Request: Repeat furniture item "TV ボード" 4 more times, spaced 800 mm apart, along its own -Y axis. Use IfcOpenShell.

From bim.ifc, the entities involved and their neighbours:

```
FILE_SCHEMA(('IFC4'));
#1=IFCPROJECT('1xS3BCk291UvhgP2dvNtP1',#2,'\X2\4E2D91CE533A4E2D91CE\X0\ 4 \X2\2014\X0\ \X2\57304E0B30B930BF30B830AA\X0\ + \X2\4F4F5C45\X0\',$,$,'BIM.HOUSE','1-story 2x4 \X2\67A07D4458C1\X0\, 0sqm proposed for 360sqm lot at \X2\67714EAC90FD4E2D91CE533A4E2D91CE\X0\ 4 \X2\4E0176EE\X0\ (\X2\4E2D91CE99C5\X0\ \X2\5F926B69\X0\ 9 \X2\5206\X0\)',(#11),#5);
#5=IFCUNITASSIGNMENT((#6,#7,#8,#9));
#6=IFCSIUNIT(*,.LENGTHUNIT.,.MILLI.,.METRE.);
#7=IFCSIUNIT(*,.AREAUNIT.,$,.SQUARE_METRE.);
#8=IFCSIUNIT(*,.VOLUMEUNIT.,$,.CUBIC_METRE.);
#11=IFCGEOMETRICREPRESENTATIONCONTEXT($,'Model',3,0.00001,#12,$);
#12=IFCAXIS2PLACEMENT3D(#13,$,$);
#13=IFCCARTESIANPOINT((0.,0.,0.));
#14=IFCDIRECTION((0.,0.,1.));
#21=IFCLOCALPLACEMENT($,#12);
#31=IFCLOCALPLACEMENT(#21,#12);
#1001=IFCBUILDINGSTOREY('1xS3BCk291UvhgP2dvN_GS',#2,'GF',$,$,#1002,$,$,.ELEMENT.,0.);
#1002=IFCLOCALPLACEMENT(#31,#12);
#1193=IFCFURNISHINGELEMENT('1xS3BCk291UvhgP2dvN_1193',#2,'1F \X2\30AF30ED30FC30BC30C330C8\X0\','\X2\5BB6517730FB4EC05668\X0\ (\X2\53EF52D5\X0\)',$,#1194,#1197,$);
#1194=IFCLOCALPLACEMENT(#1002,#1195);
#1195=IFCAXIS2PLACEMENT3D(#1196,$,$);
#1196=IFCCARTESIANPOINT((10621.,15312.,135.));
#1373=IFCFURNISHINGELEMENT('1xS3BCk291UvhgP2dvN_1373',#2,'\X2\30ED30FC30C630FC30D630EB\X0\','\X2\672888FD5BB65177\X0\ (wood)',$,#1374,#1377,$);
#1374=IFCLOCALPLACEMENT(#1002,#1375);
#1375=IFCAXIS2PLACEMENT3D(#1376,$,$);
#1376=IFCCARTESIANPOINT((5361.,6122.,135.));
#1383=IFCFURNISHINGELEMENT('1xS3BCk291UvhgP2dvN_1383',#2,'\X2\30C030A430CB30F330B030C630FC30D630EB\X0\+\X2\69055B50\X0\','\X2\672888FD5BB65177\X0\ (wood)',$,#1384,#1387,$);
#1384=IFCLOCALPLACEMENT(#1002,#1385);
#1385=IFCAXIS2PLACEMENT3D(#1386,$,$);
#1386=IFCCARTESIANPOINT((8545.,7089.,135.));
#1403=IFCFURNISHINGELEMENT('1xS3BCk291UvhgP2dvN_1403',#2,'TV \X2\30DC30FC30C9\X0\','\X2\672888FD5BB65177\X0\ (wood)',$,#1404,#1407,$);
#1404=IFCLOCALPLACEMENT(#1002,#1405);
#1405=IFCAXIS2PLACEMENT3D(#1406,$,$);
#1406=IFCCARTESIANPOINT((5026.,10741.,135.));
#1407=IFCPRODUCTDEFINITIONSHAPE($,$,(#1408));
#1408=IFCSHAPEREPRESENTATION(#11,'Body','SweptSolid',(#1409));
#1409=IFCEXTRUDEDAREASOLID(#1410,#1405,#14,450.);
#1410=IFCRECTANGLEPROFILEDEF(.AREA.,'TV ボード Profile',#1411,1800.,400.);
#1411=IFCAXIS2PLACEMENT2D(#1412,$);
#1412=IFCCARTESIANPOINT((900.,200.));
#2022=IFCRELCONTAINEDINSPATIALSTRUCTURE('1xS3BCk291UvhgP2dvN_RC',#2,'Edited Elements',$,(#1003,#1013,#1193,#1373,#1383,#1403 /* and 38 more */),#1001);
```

```python
import ifcopenshell
import ifcopenshell.api.geometry
import ifcopenshell.api.root
import ifcopenshell.util.element
import ifcopenshell.util.placement

model = ifcopenshell.open("bim.ifc")


def reuse_history(source, copy):
    """copy_class also copies each property set's owner history, people and application; keep the originals."""
    for rel in copy.IsDefinedBy:
        if rel.is_a("IfcRelDefinesByProperties") and (history := rel.RelatingPropertyDefinition.OwnerHistory):
            rel.RelatingPropertyDefinition.OwnerHistory = source.OwnerHistory
            ifcopenshell.util.element.remove_deep2(model, history)


source = model.by_id(1403)
base = ifcopenshell.util.placement.get_local_placement(source.ObjectPlacement)
step = -base[:3, 1] * 800.0

for i in range(1, 5):
    copy = ifcopenshell.api.root.copy_class(model, product=source)
    copy.Representation = ifcopenshell.util.element.copy_deep(
        model, source.Representation, exclude=["IfcGeometricRepresentationContext", "IfcRepresentationMap"]
    )
    reuse_history(source, copy)
    matrix = base.copy()
    matrix[:3, 3] += i * step
    print("added at", matrix[:3, 3].round(3) + 0.0)
    ifcopenshell.api.geometry.edit_object_placement(model, product=copy, matrix=matrix, is_si=False)

model.write("bim-out.ifc")
```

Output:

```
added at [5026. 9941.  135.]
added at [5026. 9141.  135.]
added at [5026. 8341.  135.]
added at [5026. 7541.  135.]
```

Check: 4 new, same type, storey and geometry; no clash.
